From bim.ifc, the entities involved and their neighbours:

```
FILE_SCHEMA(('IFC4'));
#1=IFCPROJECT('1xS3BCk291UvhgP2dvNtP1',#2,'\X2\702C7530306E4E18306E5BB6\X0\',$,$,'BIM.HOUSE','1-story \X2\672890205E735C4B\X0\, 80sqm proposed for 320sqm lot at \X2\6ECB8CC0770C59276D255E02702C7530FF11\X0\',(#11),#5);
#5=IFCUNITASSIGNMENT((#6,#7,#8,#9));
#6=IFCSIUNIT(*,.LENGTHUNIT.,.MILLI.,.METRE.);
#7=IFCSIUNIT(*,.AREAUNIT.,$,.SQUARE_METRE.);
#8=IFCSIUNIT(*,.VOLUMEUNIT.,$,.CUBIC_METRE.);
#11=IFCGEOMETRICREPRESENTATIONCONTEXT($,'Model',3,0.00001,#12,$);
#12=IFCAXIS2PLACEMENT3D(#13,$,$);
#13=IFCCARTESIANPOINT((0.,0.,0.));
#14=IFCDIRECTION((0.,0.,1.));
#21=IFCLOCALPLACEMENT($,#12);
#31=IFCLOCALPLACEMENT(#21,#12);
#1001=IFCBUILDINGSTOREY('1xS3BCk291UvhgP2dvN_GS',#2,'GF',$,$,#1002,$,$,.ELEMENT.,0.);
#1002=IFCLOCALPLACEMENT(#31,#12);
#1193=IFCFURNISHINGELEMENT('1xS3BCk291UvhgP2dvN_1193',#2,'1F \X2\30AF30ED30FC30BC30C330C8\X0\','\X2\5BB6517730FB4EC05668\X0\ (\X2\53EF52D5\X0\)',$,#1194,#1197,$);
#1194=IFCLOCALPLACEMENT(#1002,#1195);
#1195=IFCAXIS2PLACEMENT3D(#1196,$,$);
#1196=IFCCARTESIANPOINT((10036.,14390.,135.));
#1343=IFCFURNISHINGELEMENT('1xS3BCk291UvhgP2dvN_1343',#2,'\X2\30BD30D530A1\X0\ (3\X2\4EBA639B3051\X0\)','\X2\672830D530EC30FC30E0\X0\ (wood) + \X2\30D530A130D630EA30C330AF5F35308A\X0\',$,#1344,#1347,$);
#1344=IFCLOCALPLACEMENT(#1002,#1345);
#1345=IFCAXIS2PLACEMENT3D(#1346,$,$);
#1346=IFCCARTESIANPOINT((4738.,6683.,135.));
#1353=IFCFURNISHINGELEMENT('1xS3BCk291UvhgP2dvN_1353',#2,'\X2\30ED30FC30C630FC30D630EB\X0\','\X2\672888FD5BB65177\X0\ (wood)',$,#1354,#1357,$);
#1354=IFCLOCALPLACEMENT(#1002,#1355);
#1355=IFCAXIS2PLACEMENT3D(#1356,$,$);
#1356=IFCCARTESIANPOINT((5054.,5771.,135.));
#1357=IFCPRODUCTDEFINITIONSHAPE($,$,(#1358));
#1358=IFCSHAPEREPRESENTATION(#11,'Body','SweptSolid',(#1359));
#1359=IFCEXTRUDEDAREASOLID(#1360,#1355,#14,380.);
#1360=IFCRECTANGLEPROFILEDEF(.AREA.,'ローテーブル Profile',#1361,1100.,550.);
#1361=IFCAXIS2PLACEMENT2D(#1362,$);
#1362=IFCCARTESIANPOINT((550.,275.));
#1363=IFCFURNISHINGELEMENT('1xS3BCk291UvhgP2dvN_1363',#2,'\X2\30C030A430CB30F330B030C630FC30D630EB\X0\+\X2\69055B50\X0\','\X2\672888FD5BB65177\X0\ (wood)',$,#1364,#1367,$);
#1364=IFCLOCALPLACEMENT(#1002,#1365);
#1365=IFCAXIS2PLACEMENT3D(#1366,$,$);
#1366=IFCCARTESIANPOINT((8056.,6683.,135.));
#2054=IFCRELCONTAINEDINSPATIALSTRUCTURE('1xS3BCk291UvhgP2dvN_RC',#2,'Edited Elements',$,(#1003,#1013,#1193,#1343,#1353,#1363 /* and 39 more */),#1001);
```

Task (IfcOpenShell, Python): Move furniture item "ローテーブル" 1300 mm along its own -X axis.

```python
import ifcopenshell
import ifcopenshell.api.geometry
import ifcopenshell.util.placement
import ifcopenshell.util.unit

model = ifcopenshell.open("bim.ifc")
unit_scale = ifcopenshell.util.unit.calculate_unit_scale(model)

item = model.by_guid("1xS3BCk291UvhgP2dvN_1353")
matrix = ifcopenshell.util.placement.get_local_placement(item.ObjectPlacement)
matrix[:3, 3] -= matrix[:3, 0] * 1.3 / unit_scale
ifcopenshell.api.geometry.edit_object_placement(model, product=item, matrix=matrix, is_si=False)

print(ifcopenshell.util.placement.get_local_placement(item.ObjectPlacement).round(3) + 0.0)

model.write("bim_rev.ifc")
```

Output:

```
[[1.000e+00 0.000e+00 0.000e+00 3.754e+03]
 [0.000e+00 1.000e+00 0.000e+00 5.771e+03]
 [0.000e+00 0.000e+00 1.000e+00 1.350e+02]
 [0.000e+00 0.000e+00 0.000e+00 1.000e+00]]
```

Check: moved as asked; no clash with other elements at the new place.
